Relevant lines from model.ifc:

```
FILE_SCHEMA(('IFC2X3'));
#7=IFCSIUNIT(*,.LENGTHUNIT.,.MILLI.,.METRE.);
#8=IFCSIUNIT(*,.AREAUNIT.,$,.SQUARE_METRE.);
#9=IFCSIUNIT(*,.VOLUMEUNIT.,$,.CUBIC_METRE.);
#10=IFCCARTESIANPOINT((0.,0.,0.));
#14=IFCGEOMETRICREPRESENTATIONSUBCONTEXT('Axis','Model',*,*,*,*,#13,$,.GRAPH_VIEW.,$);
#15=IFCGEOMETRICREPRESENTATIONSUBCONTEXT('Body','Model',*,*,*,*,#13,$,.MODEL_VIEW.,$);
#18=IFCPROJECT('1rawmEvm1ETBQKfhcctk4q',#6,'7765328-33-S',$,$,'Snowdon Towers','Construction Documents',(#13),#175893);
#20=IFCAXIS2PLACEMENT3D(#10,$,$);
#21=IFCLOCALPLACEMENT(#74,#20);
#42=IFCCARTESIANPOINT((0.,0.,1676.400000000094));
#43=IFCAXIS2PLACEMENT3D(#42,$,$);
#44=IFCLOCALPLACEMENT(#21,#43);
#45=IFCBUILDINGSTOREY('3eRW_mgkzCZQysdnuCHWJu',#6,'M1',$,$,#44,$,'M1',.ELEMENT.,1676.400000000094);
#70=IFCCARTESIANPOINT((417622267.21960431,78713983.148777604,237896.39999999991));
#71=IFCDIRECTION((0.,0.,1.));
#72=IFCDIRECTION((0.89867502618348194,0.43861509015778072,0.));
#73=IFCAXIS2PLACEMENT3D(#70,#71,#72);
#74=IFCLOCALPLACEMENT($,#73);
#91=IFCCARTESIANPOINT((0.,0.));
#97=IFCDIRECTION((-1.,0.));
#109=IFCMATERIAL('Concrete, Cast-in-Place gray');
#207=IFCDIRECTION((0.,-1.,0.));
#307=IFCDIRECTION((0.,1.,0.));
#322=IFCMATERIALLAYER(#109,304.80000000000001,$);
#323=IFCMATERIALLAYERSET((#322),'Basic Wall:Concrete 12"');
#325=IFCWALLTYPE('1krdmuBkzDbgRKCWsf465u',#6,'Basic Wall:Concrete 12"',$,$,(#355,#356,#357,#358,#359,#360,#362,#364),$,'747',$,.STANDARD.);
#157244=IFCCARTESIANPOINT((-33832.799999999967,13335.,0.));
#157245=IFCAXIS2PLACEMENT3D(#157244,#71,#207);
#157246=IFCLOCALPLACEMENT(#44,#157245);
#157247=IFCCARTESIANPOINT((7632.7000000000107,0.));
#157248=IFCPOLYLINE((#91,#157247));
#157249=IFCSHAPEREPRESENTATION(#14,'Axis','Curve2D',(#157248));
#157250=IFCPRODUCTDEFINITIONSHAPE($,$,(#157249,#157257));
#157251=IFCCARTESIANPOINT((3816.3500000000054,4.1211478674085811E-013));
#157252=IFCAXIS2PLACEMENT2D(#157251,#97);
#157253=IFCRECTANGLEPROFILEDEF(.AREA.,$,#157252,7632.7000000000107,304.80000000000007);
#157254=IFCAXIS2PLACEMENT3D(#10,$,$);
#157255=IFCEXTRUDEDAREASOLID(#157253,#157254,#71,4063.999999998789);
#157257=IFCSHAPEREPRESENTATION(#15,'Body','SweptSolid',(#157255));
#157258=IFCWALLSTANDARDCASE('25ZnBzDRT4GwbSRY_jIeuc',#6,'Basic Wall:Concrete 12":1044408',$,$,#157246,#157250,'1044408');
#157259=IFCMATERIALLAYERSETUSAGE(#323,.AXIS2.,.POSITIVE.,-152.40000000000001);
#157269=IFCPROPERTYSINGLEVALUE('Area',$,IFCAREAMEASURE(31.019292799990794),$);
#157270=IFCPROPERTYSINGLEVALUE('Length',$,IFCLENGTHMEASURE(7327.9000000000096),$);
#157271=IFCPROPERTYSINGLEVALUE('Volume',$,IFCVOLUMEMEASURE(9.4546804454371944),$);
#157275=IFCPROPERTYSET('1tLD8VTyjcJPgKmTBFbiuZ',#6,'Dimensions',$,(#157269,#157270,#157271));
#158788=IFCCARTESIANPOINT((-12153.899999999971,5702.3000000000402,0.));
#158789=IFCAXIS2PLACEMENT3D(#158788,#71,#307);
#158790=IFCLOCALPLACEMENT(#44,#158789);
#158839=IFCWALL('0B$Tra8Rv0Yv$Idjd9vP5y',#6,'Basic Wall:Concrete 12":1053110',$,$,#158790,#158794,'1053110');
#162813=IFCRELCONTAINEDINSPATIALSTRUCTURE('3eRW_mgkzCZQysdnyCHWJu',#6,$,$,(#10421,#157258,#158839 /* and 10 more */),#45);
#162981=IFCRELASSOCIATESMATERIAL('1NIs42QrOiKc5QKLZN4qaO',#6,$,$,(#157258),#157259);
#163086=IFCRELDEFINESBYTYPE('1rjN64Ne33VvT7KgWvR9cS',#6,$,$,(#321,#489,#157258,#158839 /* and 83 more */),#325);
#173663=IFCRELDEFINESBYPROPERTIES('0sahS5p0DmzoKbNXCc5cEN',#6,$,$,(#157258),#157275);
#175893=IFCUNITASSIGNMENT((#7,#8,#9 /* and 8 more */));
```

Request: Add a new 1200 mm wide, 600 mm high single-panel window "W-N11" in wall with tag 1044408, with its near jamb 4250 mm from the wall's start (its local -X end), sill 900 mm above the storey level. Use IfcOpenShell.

```python
import numpy as np
import ifcopenshell
import ifcopenshell.api.feature
import ifcopenshell.api.geometry
import ifcopenshell.api.pset
import ifcopenshell.api.root
import ifcopenshell.api.spatial
import ifcopenshell.api.type
import ifcopenshell.geom
import ifcopenshell.util.element
import ifcopenshell.util.placement
import ifcopenshell.util.representation
import ifcopenshell.util.shape
import ifcopenshell.util.unit

model = ifcopenshell.open("model.ifc")
unit_scale = ifcopenshell.util.unit.calculate_unit_scale(model)
area_scale = ifcopenshell.util.unit.calculate_unit_scale(model, "AREAUNIT")
volume_scale = ifcopenshell.util.unit.calculate_unit_scale(model, "VOLUMEUNIT")
settings = ifcopenshell.geom.settings()


def volume(element):
    """Net volume in cubic metres, openings subtracted."""
    shape = ifcopenshell.geom.create_shape(settings, element)
    return ifcopenshell.util.shape.get_volume(shape.geometry)


wall = model.by_guid("25ZnBzDRT4GwbSRY_jIeuc")
storey = ifcopenshell.util.element.get_container(wall, ifc_class="IfcBuildingStorey")
context = ifcopenshell.util.representation.get_context(model, "Model", "Body", "MODEL_VIEW")
before = volume(wall)

width, height, from_end, sill = 1.2, 0.6, 4.25, 0.9  # metres

# The wall runs along its own X axis, and the end named is its -X end.
wall_shape = ifcopenshell.geom.create_shape(settings, wall)
x, y, z = ifcopenshell.util.shape.get_vertices(wall_shape.geometry).T
start = x.min() + from_end
face, thickness = float(y.min()), float(y.max() - y.min())
wall_matrix = ifcopenshell.util.placement.get_local_placement(wall.ObjectPlacement)
level = ifcopenshell.util.placement.get_local_placement(storey.ObjectPlacement)[2, 3]


def in_wall(x, y):
    """Placement at x, y metres in the wall's axes, at sill height."""
    matrix = wall_matrix.copy()
    matrix[:, 3] = wall_matrix @ np.array([x / unit_scale, y / unit_scale, 0.0, 1.0])
    matrix[2, 3] = level + sill / unit_scale
    return matrix


# Opening: a box that overshoots both wall faces by 50 mm.
opening = ifcopenshell.api.root.create_entity(model, ifc_class="IfcOpeningElement")
box = ifcopenshell.api.geometry.add_wall_representation(
    model, context=context, length=width, height=height, thickness=thickness + 0.1
)
ifcopenshell.api.geometry.assign_representation(model, product=opening, representation=box)
ifcopenshell.api.geometry.edit_object_placement(model, product=opening, matrix=in_wall(start, face - 0.05), is_si=False)
ifcopenshell.api.feature.add_feature(model, feature=opening, element=wall)

window = ifcopenshell.api.root.create_entity(model, ifc_class="IfcWindow", name="W-N11")
window.OverallWidth, window.OverallHeight = width / unit_scale, height / unit_scale
body = ifcopenshell.api.geometry.add_window_representation(
    model,
    context=context,
    overall_width=window.OverallWidth,
    overall_height=window.OverallHeight,
    partition_type="SINGLE_PANEL",
)
ifcopenshell.api.geometry.assign_representation(model, product=window, representation=body)
ifcopenshell.api.spatial.assign_container(model, products=[window], relating_structure=storey)
fills = ifcopenshell.api.feature.add_filling(model, opening=opening, element=window)
fills.OwnerHistory = window.OwnerHistory  # required in IFC2X3

# IFC2X3 keeps the operation on the window style.
style = ifcopenshell.api.root.create_entity(model, ifc_class="IfcWindowStyle", name="W-N11")
style.OperationType, style.ConstructionType = "SINGLE_PANEL", "NOTDEFINED"
style.ParameterTakesPrecedence = style.Sizeable = False
ifcopenshell.api.type.assign_type(model, related_objects=[window], relating_type=style)

# Centre the window in the wall's thickness.
ifcopenshell.api.geometry.edit_object_placement(model, product=window, matrix=in_wall(start, face), is_si=False)
window_shape = ifcopenshell.geom.create_shape(settings, window)
depth = ifcopenshell.util.shape.get_vertices(window_shape.geometry)[:, 1]
offset = face + thickness / 2 - (depth.min() + depth.max()) / 2
ifcopenshell.api.geometry.edit_object_placement(model, product=window, matrix=in_wall(start, offset), is_si=False)

after = volume(wall)

# Update the wall's stored quantities.
pset = model.by_id(ifcopenshell.util.element.get_pset(wall, "Dimensions", should_inherit=False)["id"])
ifcopenshell.api.pset.edit_pset(model, pset=pset, properties={
    "Area": model.create_entity("IfcAreaMeasure", after / thickness / area_scale),
    "Volume": model.create_entity("IfcVolumeMeasure", after / volume_scale),
})

print(f"wall volume {before:.3f} -> {after:.3f} m3")

model.write("model-out.ifc")
```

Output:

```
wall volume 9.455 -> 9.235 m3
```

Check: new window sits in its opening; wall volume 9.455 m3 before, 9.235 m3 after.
